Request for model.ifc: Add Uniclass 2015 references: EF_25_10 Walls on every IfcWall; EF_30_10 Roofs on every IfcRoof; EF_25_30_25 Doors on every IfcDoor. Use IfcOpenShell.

First a look at what the model holds.

```python
import ifcopenshell

model = ifcopenshell.open("model.ifc")
print(model.schema)
print("classifications:", [c.Name for c in model.by_type("IfcClassification")])
for ifc_class in ("IfcDoor", "IfcRoof", "IfcStair", "IfcWall", "IfcWindow"):
    print(ifc_class, len(model.by_type(ifc_class)))
```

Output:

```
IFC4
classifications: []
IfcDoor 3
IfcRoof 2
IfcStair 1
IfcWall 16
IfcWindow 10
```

```python
import ifcopenshell
import ifcopenshell.api.classification

model = ifcopenshell.open("model.ifc")

system = ifcopenshell.api.classification.add_classification(model, classification="Uniclass 2015")

codes = {
    "IfcWall": ("EF_25_10", "Walls"),
    "IfcRoof": ("EF_30_10", "Roofs"),
    "IfcDoor": ("EF_25_30_25", "Doors"),
}
for ifc_class, (code, name) in codes.items():
    products = model.by_type(ifc_class)
    ifcopenshell.api.classification.add_reference(
        model, products=products, classification=system, identification=code, name=name
    )
    print(code, len(products))

model.write("model_v2.ifc")
```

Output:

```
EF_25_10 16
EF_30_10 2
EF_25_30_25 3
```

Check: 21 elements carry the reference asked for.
